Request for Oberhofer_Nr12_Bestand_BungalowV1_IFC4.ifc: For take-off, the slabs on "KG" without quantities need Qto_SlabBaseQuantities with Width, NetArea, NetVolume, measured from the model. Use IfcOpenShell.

First a look at what the model holds.

```python
import ifcopenshell
import ifcopenshell.util.element
import ifcopenshell.util.unit

model = ifcopenshell.open("Oberhofer_Nr12_Bestand_BungalowV1_IFC4.ifc")
print(model.schema)
for unit_type in ("LENGTHUNIT", "AREAUNIT", "VOLUMEUNIT"):
    print(unit_type, ifcopenshell.util.unit.calculate_unit_scale(model, unit_type))
storey = next(s for s in model.by_type("IfcBuildingStorey") if s.Name == "KG")
slabs = [e for e in ifcopenshell.util.element.get_decomposition(storey) if e.is_a("IfcSlab")]
for e in sorted(slabs, key=lambda e: e.id()):
    print(e.id(), e.is_a(), e.Name, list(ifcopenshell.util.element.get_psets(e, qtos_only=True)), sep=" | ")
```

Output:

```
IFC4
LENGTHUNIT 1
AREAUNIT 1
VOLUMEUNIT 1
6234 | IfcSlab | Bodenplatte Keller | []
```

```python
import ifcopenshell
import ifcopenshell.api.pset
import ifcopenshell.geom
import ifcopenshell.util.element
import ifcopenshell.util.shape
import ifcopenshell.util.unit

model = ifcopenshell.open("Oberhofer_Nr12_Bestand_BungalowV1_IFC4.ifc")
unit_scale = ifcopenshell.util.unit.calculate_unit_scale(model)
area_scale = ifcopenshell.util.unit.calculate_unit_scale(model, "AREAUNIT")
volume_scale = ifcopenshell.util.unit.calculate_unit_scale(model, "VOLUMEUNIT")
settings = ifcopenshell.geom.settings()

storey = next(s for s in model.by_type("IfcBuildingStorey") if s.Name == "KG")
slabs = [e for e in ifcopenshell.util.element.get_decomposition(storey) if e.is_a("IfcSlab")]

for e in sorted(slabs, key=lambda e: e.id()):
    if ifcopenshell.util.element.get_psets(e, qtos_only=True, should_inherit=False):
        continue
    # Geometry comes back in metres, in the element's own axes.
    shape = ifcopenshell.geom.create_shape(settings, e)
    values = {
        "Width": ifcopenshell.util.shape.get_z(shape.geometry) / unit_scale,
        "NetArea": ifcopenshell.util.shape.get_footprint_area(shape.geometry) / area_scale,
        "NetVolume": ifcopenshell.util.shape.get_volume(shape.geometry) / volume_scale,
    }
    qto = ifcopenshell.api.pset.add_qto(model, product=e, name="Qto_SlabBaseQuantities")
    ifcopenshell.api.pset.edit_qto(model, qto=qto, properties=values)
    print(e.id(), {k: round(v, 3) for k, v in values.items()})

model.write("Oberhofer_Nr12_Bestand_BungalowV1_IFC4_edited.ifc")
```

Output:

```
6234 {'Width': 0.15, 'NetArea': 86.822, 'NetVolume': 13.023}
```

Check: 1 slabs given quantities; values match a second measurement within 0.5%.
